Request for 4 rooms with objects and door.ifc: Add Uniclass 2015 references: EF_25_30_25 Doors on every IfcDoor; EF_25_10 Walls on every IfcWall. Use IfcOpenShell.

First a look at what the model holds.

```python
import ifcopenshell

model = ifcopenshell.open("4 rooms with objects and door.ifc")
print(model.schema)
print("classifications:", [c.Name for c in model.by_type("IfcClassification")])
for ifc_class in ("IfcDoor", "IfcRoof", "IfcStair", "IfcWall", "IfcWindow"):
    print(ifc_class, len(model.by_type(ifc_class)))
```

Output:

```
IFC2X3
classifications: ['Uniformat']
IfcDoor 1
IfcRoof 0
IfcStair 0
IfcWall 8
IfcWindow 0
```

```python
import ifcopenshell
import ifcopenshell.api.classification

model = ifcopenshell.open("4 rooms with objects and door.ifc")

# IFC2X3 requires Source and Edition and has no link from the project to the system.
system = model.create_entity("IfcClassification", Source="NBS", Edition="2015", Name="Uniclass 2015")

codes = {
    "IfcDoor": ("EF_25_30_25", "Doors"),
    "IfcWall": ("EF_25_10", "Walls"),
}
for ifc_class, (code, name) in codes.items():
    products = model.by_type(ifc_class)
    ifcopenshell.api.classification.add_reference(
        model, products=products, classification=system, identification=code, name=name
    )
    print(code, len(products))

model.write("4 rooms with objects and door_edited.ifc")
```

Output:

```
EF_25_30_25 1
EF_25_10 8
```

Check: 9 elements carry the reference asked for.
